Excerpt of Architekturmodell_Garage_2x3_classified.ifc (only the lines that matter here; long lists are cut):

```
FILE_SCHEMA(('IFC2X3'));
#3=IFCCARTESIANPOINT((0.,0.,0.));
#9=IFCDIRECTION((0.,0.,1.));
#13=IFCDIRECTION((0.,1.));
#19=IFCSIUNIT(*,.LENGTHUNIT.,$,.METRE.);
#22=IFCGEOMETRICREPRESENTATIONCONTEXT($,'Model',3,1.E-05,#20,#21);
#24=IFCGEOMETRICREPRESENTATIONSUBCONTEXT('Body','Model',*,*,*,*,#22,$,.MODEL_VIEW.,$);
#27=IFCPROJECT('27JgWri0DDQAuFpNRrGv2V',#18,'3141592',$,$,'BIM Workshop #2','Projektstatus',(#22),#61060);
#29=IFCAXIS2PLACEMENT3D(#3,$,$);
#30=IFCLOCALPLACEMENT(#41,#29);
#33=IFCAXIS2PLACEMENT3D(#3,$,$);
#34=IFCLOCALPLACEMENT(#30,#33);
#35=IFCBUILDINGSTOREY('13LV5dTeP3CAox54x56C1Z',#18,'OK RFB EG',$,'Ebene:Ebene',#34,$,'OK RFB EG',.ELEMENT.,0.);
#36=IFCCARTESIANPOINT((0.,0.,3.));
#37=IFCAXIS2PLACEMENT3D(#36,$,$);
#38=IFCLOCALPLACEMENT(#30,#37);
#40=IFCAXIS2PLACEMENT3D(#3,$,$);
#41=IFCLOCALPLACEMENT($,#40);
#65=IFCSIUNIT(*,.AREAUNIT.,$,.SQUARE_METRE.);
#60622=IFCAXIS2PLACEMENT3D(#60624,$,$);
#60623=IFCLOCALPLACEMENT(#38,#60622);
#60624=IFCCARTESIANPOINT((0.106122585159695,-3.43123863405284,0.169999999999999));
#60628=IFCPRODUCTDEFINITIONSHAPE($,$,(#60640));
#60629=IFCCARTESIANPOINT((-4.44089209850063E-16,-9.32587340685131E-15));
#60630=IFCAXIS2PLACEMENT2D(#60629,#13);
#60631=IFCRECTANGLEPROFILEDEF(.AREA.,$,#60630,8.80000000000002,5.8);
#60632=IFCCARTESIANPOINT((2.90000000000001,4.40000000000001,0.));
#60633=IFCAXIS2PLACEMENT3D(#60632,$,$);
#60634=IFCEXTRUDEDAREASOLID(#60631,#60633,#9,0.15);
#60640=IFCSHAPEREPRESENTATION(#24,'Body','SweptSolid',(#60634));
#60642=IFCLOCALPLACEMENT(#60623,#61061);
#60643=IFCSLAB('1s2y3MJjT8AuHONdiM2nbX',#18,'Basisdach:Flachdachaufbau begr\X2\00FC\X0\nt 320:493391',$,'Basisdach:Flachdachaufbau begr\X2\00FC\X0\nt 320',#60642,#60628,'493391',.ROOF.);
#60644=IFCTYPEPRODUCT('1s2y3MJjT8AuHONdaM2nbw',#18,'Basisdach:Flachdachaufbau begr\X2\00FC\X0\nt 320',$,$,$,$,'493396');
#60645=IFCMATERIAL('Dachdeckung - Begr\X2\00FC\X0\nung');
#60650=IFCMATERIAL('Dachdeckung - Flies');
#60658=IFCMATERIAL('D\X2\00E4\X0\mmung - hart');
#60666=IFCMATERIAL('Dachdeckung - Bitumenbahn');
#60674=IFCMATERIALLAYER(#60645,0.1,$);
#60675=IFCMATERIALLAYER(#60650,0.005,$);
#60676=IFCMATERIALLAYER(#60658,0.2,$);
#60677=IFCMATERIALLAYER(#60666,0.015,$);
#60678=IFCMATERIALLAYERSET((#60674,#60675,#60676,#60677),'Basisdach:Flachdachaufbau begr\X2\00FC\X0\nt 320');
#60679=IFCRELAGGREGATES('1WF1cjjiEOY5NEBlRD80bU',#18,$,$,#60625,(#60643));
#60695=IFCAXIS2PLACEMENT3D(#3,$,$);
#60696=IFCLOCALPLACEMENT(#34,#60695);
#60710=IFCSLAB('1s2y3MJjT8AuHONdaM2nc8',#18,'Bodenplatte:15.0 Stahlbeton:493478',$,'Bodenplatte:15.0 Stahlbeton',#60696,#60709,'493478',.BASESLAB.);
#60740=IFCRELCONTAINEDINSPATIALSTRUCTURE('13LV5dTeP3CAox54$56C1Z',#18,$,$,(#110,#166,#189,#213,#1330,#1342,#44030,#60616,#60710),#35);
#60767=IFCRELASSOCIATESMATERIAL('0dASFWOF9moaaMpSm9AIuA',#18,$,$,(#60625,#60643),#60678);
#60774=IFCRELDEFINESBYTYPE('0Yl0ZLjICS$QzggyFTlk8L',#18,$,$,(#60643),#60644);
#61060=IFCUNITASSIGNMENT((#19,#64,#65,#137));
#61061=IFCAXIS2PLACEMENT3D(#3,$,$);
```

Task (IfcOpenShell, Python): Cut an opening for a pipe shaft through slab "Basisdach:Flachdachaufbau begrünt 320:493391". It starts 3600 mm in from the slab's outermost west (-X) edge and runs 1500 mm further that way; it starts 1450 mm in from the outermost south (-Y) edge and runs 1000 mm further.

```python
import numpy as np
import ifcopenshell
import ifcopenshell.api.feature
import ifcopenshell.api.geometry
import ifcopenshell.api.root
import ifcopenshell.geom
import ifcopenshell.util.placement
import ifcopenshell.util.representation
import ifcopenshell.util.shape
import ifcopenshell.util.unit

model = ifcopenshell.open("Architekturmodell_Garage_2x3_classified.ifc")
unit_scale = ifcopenshell.util.unit.calculate_unit_scale(model)
settings = ifcopenshell.geom.settings()


def volume(element):
    """Net volume in cubic metres, openings subtracted."""
    shape = ifcopenshell.geom.create_shape(settings, element)
    return ifcopenshell.util.shape.get_volume(shape.geometry)


slab = model.by_guid("1s2y3MJjT8AuHONdiM2nbX")
before = volume(slab)

# Extent in the slab's own axes, in metres. The edges named are its -X and -Y sides.
slab_shape = ifcopenshell.geom.create_shape(settings, slab)
vertices = ifcopenshell.util.shape.get_vertices(slab_shape.geometry)
x_min, y_min, bottom = vertices.min(axis=0)
top = vertices[:, 2].max()

opening = ifcopenshell.api.root.create_entity(model, ifc_class="IfcOpeningElement", name="Pipe shaft opening")
context = ifcopenshell.util.representation.get_context(model, "Model", "Body", "MODEL_VIEW")
width, depth = 1.5, 1
outline = [(0.0, 0.0), (width, 0.0), (width, depth), (0.0, depth), (0.0, 0.0)]
# Overshoot both faces by 50 mm so the cut is clean.
shape = ifcopenshell.api.geometry.add_slab_representation(
    model, context=context, depth=top - bottom + 0.1, polyline=outline
)
ifcopenshell.api.geometry.assign_representation(model, product=opening, representation=shape)

matrix = ifcopenshell.util.placement.get_local_placement(slab.ObjectPlacement)
matrix[:, 3] = matrix @ np.append(np.array([x_min + 3.6, y_min + 1.45, bottom - 0.05]) / unit_scale, 1.0)
ifcopenshell.api.geometry.edit_object_placement(model, product=opening, matrix=matrix, is_si=False)
ifcopenshell.api.feature.add_feature(model, feature=opening, element=slab)

after = volume(slab)

print(f"slab volume {before:.3f} -> {after:.3f} m3")

model.write("Architekturmodell_Garage_2x3_classified_v2.ifc")
```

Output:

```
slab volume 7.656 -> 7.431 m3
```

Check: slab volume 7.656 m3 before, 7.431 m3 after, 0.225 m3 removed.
